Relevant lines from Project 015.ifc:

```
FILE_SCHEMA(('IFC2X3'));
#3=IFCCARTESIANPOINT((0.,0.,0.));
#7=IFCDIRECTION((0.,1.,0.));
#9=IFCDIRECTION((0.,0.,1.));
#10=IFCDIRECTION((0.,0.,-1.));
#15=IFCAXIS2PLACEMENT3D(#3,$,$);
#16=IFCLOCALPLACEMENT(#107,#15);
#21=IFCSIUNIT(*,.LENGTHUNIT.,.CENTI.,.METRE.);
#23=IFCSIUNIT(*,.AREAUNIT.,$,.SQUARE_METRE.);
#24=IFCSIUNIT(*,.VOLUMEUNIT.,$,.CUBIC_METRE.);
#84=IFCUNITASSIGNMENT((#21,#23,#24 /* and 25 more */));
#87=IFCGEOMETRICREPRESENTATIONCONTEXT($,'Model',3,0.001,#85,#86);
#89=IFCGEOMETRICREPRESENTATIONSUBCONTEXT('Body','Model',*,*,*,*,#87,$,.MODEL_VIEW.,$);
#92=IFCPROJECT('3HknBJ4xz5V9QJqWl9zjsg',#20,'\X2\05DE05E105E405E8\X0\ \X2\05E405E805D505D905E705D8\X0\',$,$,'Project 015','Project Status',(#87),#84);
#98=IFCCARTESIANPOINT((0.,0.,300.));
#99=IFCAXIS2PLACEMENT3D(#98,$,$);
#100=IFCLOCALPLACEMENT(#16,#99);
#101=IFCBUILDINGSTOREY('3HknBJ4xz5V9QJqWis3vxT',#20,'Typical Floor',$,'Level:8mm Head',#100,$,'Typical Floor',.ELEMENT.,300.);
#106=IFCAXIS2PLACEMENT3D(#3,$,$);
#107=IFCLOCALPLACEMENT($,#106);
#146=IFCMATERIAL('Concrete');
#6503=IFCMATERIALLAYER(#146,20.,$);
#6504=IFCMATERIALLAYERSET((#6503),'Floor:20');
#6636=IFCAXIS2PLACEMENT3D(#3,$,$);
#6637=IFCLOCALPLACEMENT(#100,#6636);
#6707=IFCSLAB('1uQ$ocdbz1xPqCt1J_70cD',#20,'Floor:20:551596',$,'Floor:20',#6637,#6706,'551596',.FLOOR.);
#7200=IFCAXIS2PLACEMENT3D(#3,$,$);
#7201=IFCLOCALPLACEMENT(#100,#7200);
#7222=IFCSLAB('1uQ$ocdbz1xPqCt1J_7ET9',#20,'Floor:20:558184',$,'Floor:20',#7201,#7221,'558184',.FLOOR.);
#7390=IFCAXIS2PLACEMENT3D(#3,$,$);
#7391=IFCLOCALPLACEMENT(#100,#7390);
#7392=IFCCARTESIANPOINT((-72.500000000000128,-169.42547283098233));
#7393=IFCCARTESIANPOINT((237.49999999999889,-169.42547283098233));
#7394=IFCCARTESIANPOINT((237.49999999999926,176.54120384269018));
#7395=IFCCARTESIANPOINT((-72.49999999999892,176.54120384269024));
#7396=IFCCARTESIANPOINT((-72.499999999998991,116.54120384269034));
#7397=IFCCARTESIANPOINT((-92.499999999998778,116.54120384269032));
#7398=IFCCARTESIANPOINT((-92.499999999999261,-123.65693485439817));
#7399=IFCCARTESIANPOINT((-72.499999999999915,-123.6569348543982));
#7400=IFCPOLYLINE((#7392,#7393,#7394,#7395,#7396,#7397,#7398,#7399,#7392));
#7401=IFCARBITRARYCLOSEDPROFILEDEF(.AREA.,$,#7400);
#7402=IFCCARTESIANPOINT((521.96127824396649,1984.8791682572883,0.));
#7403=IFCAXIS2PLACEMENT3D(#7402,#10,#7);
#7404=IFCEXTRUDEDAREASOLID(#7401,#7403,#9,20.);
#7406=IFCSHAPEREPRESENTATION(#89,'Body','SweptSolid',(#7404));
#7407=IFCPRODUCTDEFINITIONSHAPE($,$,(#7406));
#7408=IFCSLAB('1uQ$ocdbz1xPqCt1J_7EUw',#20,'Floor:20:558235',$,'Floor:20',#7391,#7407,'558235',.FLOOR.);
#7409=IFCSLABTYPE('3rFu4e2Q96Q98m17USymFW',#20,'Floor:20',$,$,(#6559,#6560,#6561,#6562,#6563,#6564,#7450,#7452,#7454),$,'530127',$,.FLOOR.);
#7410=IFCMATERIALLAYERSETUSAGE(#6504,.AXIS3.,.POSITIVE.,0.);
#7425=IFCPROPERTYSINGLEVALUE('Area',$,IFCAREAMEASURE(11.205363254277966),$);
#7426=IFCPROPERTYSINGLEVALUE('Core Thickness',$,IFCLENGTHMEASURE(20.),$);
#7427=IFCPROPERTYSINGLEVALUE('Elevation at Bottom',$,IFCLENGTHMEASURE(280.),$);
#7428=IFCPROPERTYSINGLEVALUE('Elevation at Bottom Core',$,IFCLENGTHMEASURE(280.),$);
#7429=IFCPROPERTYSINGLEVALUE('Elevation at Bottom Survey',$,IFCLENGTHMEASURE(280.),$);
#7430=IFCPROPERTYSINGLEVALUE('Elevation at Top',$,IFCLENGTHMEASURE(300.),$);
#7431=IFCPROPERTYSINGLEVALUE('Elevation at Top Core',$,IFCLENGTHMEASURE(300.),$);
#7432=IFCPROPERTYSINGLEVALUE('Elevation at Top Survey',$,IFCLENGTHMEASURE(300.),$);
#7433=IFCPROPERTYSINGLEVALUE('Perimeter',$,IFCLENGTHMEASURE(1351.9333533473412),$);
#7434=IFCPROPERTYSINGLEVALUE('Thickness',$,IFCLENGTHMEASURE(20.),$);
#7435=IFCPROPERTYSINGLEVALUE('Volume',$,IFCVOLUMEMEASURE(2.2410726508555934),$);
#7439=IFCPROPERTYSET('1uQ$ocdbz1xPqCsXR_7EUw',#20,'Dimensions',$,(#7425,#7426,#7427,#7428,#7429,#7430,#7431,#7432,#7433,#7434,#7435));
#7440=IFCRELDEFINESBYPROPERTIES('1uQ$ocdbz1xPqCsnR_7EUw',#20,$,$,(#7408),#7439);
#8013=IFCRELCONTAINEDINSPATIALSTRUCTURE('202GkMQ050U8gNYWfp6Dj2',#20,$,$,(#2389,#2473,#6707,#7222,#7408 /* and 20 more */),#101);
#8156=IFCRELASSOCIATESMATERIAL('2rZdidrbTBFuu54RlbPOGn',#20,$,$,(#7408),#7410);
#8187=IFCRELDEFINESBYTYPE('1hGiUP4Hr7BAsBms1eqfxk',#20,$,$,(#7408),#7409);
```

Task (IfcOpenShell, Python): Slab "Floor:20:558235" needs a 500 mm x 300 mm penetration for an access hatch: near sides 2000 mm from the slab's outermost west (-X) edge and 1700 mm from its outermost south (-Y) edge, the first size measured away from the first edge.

```python
import numpy as np
import ifcopenshell
import ifcopenshell.api.feature
import ifcopenshell.api.geometry
import ifcopenshell.api.pset
import ifcopenshell.api.root
import ifcopenshell.geom
import ifcopenshell.util.element
import ifcopenshell.util.placement
import ifcopenshell.util.representation
import ifcopenshell.util.shape
import ifcopenshell.util.unit

model = ifcopenshell.open("Project 015.ifc")
unit_scale = ifcopenshell.util.unit.calculate_unit_scale(model)
area_scale = ifcopenshell.util.unit.calculate_unit_scale(model, "AREAUNIT")
volume_scale = ifcopenshell.util.unit.calculate_unit_scale(model, "VOLUMEUNIT")
settings = ifcopenshell.geom.settings()


def volume(element):
    """Net volume in cubic metres, openings subtracted."""
    shape = ifcopenshell.geom.create_shape(settings, element)
    return ifcopenshell.util.shape.get_volume(shape.geometry)


slab = model.by_guid("1uQ$ocdbz1xPqCt1J_7EUw")
before = volume(slab)

# Extent in the slab's own axes, in metres. The edges named are its -X and -Y sides.
slab_shape = ifcopenshell.geom.create_shape(settings, slab)
vertices = ifcopenshell.util.shape.get_vertices(slab_shape.geometry)
x_min, y_min, bottom = vertices.min(axis=0)
top = vertices[:, 2].max()

opening = ifcopenshell.api.root.create_entity(model, ifc_class="IfcOpeningElement", name="Access hatch opening")
context = ifcopenshell.util.representation.get_context(model, "Model", "Body", "MODEL_VIEW")
width, depth = 0.5, 0.3
outline = [(0.0, 0.0), (width, 0.0), (width, depth), (0.0, depth), (0.0, 0.0)]
# Overshoot both faces by 50 mm so the cut is clean.
shape = ifcopenshell.api.geometry.add_slab_representation(
    model, context=context, depth=top - bottom + 0.1, polyline=outline
)
ifcopenshell.api.geometry.assign_representation(model, product=opening, representation=shape)

matrix = ifcopenshell.util.placement.get_local_placement(slab.ObjectPlacement)
matrix[:, 3] = matrix @ np.append(np.array([x_min + 2, y_min + 1.7, bottom - 0.05]) / unit_scale, 1.0)
ifcopenshell.api.geometry.edit_object_placement(model, product=opening, matrix=matrix, is_si=False)
ifcopenshell.api.feature.add_feature(model, feature=opening, element=slab)

after = volume(slab)

# Update the slab's stored quantities.
pset = model.by_id(ifcopenshell.util.element.get_pset(slab, "Dimensions", should_inherit=False)["id"])
ifcopenshell.api.pset.edit_pset(model, pset=pset, properties={
    "Area": model.create_entity("IfcAreaMeasure", after / (top - bottom) / area_scale),
    "Volume": model.create_entity("IfcVolumeMeasure", after / volume_scale),
})

print(f"slab volume {before:.3f} -> {after:.3f} m3")

model.write("Project 015_rev.ifc")
```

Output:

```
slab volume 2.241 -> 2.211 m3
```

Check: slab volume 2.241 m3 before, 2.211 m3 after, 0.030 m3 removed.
